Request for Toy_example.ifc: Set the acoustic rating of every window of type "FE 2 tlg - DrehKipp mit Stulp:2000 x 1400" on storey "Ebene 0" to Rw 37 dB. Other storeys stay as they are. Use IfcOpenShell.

First a look at what the model holds.

```python
import ifcopenshell
import ifcopenshell.util.element

model = ifcopenshell.open("Toy_example.ifc")
print(model.schema)
storey = next(s for s in model.by_type("IfcBuildingStorey") if s.Name == "Ebene 0")
windows = [e for e in ifcopenshell.util.element.get_decomposition(storey) if e.is_a("IfcWindow")]
seen = {}
for e in windows:
    element_type = ifcopenshell.util.element.get_type(e)
    key = (element_type.Name if element_type != e and element_type else None, ifcopenshell.util.element.get_pset(e, "Pset_WindowCommon", "AcousticRating"))
    seen[key] = seen.get(key, 0) + 1
for (name, value), count in sorted(seen.items(), key=str):
    print(count, "x", name, "|", value)
```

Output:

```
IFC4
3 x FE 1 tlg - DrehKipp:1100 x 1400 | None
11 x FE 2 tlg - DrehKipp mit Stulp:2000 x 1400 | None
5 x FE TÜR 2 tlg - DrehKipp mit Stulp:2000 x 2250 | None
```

```python
import ifcopenshell
import ifcopenshell.api.pset
import ifcopenshell.util.element

model = ifcopenshell.open("Toy_example.ifc")

storey = next(s for s in model.by_type("IfcBuildingStorey") if s.Name == "Ebene 0")
windows = [e for e in ifcopenshell.util.element.get_decomposition(storey) if e.is_a("IfcWindow")]

count = 0
for e in windows:
    element_type = ifcopenshell.util.element.get_type(e)
    if element_type in (None, e) or element_type.Name != "FE 2 tlg - DrehKipp mit Stulp:2000 x 1400":
        continue
    # add_pset returns the element's existing set when there is one.
    pset = ifcopenshell.api.pset.add_pset(model, product=e, name="Pset_WindowCommon")
    ifcopenshell.api.pset.edit_pset(model, pset=pset, properties={"AcousticRating": "Rw 37 dB"})
    count += 1

print(count, "windows updated")

model.write("Toy_example_rev.ifc")
```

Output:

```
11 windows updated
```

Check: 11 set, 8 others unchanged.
